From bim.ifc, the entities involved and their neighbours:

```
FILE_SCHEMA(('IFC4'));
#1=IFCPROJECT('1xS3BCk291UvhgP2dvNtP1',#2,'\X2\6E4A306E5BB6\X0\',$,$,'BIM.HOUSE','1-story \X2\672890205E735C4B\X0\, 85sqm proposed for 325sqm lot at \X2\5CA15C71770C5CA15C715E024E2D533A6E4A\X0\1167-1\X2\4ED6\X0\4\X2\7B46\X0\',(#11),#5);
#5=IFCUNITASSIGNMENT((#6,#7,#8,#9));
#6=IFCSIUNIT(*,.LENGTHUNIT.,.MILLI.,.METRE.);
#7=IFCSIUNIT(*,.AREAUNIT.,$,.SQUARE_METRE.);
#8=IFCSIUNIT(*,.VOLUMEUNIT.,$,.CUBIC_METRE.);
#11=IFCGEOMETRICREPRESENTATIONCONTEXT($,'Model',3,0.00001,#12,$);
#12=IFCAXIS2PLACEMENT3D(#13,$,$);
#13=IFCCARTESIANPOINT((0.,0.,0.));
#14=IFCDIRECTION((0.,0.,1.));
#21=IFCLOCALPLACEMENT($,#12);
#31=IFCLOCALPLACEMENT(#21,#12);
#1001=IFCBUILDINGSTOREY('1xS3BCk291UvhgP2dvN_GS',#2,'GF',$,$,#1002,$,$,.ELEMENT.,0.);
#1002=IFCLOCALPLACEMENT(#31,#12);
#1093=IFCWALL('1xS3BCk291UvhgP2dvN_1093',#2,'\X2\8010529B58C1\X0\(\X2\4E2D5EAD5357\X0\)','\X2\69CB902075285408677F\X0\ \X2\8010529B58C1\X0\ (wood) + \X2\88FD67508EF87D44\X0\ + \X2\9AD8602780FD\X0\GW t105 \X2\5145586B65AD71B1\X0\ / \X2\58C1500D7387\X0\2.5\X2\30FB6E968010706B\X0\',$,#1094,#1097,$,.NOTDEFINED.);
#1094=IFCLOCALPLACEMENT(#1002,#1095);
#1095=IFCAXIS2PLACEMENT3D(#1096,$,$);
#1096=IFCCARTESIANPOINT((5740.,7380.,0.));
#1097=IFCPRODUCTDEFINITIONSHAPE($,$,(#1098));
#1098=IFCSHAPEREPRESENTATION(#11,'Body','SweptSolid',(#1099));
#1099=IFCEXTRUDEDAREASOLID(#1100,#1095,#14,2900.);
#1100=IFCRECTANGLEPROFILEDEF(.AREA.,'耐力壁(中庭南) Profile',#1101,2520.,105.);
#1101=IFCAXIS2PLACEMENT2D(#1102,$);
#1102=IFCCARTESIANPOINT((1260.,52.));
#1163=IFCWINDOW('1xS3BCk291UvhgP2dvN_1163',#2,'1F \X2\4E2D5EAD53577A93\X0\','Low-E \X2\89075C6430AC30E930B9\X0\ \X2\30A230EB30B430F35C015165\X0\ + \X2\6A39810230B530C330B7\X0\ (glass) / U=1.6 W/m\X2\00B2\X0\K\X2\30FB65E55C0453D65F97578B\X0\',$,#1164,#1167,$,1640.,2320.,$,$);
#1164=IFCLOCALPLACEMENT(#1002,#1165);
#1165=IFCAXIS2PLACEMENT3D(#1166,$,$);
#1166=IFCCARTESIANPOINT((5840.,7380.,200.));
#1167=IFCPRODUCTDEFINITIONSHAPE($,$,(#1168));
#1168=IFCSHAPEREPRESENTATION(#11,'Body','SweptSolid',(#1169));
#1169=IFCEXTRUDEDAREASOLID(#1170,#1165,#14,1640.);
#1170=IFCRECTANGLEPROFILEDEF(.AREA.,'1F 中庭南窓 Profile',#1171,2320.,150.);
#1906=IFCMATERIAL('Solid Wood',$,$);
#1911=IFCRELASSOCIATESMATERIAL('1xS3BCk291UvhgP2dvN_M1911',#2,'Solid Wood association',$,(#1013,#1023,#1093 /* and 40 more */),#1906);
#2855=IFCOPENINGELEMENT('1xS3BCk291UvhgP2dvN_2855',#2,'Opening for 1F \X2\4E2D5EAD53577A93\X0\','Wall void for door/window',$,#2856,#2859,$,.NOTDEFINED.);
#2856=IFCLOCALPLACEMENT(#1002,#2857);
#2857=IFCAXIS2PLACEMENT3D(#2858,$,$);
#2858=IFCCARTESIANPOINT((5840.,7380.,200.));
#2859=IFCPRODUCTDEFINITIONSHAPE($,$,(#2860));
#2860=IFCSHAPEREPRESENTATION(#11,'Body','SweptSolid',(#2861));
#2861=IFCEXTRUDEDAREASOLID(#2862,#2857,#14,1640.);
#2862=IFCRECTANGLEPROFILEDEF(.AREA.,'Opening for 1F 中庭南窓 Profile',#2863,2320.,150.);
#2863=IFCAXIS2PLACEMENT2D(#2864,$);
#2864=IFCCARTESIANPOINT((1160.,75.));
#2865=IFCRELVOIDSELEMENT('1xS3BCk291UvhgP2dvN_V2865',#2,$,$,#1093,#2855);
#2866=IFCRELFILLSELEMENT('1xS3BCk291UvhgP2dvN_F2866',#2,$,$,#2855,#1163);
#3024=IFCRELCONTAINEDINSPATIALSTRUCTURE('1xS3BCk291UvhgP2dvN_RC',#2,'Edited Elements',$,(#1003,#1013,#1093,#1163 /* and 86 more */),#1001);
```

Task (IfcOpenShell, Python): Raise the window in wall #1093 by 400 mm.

```python
import numpy as np
import ifcopenshell
import ifcopenshell.api.geometry
import ifcopenshell.util.placement
import ifcopenshell.util.unit

model = ifcopenshell.open("bim.ifc")
unit_scale = ifcopenshell.util.unit.calculate_unit_scale(model)

window = model.by_guid("1xS3BCk291UvhgP2dvN_1163")
opening = window.FillsVoids[0].RelatingOpeningElement
dz = 400.0

shift = np.array([0.0, 0.0, dz])
# The window is not placed relative to its opening, so move both.
for product in (opening, window):
    matrix = ifcopenshell.util.placement.get_local_placement(product.ObjectPlacement)
    matrix[:3, 3] += shift
    ifcopenshell.api.geometry.edit_object_placement(model, product=product, matrix=matrix, is_si=False)

print(f"moved by {dz * unit_scale:+.3f} m")

model.write("bim_updated.ifc")
```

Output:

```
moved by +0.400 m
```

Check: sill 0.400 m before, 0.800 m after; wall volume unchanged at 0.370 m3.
